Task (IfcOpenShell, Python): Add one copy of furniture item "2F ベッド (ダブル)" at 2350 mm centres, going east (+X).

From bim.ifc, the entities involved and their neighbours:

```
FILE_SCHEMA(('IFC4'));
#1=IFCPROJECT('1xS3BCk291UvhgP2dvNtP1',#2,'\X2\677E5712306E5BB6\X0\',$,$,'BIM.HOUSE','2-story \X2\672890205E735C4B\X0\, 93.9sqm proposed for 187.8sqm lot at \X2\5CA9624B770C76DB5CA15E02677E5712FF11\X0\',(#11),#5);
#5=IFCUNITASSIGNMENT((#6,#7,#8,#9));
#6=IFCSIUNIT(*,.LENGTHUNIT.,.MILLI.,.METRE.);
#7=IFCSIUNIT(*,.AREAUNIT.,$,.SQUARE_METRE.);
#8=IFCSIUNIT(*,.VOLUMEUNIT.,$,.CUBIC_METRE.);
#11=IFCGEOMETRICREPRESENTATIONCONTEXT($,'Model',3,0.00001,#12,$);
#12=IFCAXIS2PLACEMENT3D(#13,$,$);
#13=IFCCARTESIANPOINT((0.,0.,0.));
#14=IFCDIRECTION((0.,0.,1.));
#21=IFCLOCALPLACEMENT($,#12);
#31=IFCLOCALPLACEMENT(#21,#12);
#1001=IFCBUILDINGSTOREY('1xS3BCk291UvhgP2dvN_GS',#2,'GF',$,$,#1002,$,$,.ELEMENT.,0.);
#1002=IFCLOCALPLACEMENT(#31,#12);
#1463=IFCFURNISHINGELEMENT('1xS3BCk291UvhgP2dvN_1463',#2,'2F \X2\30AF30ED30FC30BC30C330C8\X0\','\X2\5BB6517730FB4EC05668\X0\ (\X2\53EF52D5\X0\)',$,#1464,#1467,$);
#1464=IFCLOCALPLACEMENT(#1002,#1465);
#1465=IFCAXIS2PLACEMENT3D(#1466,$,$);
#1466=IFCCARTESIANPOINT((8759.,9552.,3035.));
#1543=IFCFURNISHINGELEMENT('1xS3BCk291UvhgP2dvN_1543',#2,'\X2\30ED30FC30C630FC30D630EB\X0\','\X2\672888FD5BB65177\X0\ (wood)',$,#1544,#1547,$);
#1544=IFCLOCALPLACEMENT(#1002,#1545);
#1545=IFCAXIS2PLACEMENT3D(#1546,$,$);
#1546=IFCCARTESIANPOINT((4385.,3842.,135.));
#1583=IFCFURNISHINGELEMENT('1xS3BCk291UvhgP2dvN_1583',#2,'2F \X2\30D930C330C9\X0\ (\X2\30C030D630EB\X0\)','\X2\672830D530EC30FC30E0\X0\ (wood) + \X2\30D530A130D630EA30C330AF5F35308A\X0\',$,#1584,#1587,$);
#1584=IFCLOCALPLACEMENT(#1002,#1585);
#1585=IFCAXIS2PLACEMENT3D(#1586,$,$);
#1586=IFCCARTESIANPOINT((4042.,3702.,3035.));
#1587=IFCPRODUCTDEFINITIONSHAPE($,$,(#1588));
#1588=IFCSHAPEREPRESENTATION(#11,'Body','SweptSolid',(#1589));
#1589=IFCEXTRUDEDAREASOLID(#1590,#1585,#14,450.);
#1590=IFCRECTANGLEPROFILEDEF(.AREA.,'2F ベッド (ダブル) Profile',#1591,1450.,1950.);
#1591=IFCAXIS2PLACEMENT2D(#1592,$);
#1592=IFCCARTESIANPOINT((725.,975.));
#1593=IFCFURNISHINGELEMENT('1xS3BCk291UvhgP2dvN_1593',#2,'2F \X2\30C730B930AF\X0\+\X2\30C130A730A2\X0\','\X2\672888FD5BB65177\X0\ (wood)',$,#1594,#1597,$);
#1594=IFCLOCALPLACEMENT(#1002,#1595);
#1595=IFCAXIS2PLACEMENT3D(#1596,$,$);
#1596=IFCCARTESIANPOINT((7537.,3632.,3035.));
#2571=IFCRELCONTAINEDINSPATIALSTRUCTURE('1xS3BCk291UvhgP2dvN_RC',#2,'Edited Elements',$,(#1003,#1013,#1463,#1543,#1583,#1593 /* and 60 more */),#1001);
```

```python
import numpy as np
import ifcopenshell
import ifcopenshell.api.geometry
import ifcopenshell.api.root
import ifcopenshell.util.element
import ifcopenshell.util.placement

model = ifcopenshell.open("bim.ifc")


def reuse_history(source, copy):
    """copy_class also copies each property set's owner history, people and application; keep the originals."""
    for rel in copy.IsDefinedBy:
        if rel.is_a("IfcRelDefinesByProperties") and (history := rel.RelatingPropertyDefinition.OwnerHistory):
            rel.RelatingPropertyDefinition.OwnerHistory = source.OwnerHistory
            ifcopenshell.util.element.remove_deep2(model, history)


source = model.by_guid("1xS3BCk291UvhgP2dvN_1583")
base = ifcopenshell.util.placement.get_local_placement(source.ObjectPlacement)
step = np.array([1.0, 0.0, 0.0]) * 2350.0

for i in range(1, 2):
    copy = ifcopenshell.api.root.copy_class(model, product=source)
    copy.Representation = ifcopenshell.util.element.copy_deep(
        model, source.Representation, exclude=["IfcGeometricRepresentationContext", "IfcRepresentationMap"]
    )
    reuse_history(source, copy)
    matrix = base.copy()
    matrix[:3, 3] += i * step
    print("added at", matrix[:3, 3].round(3) + 0.0)
    ifcopenshell.api.geometry.edit_object_placement(model, product=copy, matrix=matrix, is_si=False)

model.write("bim_v2.ifc")
```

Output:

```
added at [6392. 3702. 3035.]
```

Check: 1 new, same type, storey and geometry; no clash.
